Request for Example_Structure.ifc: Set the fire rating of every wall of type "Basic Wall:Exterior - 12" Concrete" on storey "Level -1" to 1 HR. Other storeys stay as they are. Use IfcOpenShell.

First a look at what the model holds.

```python
import ifcopenshell
import ifcopenshell.util.element

model = ifcopenshell.open("Example_Structure.ifc")
print(model.schema)
storey = next(s for s in model.by_type("IfcBuildingStorey") if s.Name == "Level -1")
walls = [e for e in ifcopenshell.util.element.get_decomposition(storey) if e.is_a("IfcWall")]
seen = {}
for e in walls:
    element_type = ifcopenshell.util.element.get_type(e)
    key = (element_type.Name if element_type != e and element_type else None, ifcopenshell.util.element.get_pset(e, "Pset_WallCommon", "FireRating"))
    seen[key] = seen.get(key, 0) + 1
for (name, value), count in sorted(seen.items(), key=str):
    print(count, "x", name, "|", value)
```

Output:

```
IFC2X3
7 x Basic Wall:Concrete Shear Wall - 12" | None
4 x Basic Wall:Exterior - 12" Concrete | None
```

```python
import ifcopenshell
import ifcopenshell.api.pset
import ifcopenshell.util.element

model = ifcopenshell.open("Example_Structure.ifc")

storey = next(s for s in model.by_type("IfcBuildingStorey") if s.Name == "Level -1")
walls = [e for e in ifcopenshell.util.element.get_decomposition(storey) if e.is_a("IfcWall")]

count = 0
for e in walls:
    element_type = ifcopenshell.util.element.get_type(e)
    if element_type in (None, e) or element_type.Name != 'Basic Wall:Exterior - 12" Concrete':
        continue
    # add_pset returns the element's existing set when there is one.
    pset = ifcopenshell.api.pset.add_pset(model, product=e, name="Pset_WallCommon")
    ifcopenshell.api.pset.edit_pset(model, pset=pset, properties={"FireRating": "1 HR"})
    count += 1

print(count, "walls updated")

model.write("Example_Structure_updated.ifc")
```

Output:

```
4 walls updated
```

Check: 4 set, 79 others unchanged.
